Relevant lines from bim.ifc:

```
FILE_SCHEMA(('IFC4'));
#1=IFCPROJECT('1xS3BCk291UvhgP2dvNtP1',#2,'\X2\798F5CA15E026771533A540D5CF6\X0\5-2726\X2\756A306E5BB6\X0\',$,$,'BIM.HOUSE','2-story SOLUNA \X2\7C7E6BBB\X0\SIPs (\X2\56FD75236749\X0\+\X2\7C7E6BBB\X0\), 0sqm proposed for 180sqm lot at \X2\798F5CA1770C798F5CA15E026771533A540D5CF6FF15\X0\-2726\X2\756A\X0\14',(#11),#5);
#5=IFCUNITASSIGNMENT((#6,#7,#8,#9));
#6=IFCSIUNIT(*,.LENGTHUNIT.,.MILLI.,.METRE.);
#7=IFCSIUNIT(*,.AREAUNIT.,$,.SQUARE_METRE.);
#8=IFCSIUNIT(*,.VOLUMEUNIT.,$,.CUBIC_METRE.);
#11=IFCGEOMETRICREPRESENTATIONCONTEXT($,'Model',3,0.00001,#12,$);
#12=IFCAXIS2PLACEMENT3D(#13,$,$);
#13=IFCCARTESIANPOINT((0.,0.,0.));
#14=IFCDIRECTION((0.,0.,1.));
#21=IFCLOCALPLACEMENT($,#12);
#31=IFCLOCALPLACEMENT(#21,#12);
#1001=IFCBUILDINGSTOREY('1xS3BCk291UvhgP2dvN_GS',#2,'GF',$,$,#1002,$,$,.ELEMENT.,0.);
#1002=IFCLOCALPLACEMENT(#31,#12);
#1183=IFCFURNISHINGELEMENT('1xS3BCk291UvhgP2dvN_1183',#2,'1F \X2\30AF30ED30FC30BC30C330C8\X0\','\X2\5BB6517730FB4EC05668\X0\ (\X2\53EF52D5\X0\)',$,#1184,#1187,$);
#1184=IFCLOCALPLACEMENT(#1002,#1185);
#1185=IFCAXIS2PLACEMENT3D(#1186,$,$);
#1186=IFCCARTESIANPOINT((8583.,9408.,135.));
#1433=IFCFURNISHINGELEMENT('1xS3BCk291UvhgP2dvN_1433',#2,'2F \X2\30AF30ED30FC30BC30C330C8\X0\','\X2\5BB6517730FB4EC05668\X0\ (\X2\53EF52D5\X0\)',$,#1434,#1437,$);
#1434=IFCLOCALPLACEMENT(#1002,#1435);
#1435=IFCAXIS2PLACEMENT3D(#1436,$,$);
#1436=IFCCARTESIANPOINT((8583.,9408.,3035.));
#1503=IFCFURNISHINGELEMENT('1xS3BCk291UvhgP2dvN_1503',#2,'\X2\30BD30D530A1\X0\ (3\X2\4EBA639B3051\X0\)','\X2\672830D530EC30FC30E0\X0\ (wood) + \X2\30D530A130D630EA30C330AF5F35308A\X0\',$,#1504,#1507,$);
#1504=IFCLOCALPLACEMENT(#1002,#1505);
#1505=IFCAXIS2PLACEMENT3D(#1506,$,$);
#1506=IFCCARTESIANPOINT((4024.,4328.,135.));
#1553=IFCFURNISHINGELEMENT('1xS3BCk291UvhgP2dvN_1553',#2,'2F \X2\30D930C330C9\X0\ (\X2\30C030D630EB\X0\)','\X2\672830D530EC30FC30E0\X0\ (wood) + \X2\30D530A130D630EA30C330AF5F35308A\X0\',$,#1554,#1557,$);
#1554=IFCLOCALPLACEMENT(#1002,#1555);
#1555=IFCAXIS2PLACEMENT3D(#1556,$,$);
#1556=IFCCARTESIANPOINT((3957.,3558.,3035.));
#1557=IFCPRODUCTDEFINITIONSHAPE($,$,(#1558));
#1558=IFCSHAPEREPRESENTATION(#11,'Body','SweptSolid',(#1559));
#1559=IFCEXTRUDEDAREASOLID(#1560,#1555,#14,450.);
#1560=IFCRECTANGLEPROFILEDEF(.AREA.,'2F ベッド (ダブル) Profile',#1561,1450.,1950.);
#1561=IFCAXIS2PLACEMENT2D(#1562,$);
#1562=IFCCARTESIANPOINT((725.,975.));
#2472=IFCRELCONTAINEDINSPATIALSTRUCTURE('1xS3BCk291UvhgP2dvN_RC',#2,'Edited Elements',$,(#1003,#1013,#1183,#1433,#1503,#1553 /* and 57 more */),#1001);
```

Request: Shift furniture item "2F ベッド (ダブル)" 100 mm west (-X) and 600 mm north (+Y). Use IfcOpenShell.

```python
import ifcopenshell
import ifcopenshell.api.geometry
import ifcopenshell.util.placement
import ifcopenshell.util.unit

model = ifcopenshell.open("bim.ifc")
unit_scale = ifcopenshell.util.unit.calculate_unit_scale(model)

item = model.by_guid("1xS3BCk291UvhgP2dvN_1553")
matrix = ifcopenshell.util.placement.get_local_placement(item.ObjectPlacement)
matrix[0, 3] -= 0.1 / unit_scale
matrix[1, 3] += 0.6 / unit_scale
ifcopenshell.api.geometry.edit_object_placement(model, product=item, matrix=matrix, is_si=False)

print(ifcopenshell.util.placement.get_local_placement(item.ObjectPlacement).round(3) + 0.0)

model.write("bim-out.ifc")
```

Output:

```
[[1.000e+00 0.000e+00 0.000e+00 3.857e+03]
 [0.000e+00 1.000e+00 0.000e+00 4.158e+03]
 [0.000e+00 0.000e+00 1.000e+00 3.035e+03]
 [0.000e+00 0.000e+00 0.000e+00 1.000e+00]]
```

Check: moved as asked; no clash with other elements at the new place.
